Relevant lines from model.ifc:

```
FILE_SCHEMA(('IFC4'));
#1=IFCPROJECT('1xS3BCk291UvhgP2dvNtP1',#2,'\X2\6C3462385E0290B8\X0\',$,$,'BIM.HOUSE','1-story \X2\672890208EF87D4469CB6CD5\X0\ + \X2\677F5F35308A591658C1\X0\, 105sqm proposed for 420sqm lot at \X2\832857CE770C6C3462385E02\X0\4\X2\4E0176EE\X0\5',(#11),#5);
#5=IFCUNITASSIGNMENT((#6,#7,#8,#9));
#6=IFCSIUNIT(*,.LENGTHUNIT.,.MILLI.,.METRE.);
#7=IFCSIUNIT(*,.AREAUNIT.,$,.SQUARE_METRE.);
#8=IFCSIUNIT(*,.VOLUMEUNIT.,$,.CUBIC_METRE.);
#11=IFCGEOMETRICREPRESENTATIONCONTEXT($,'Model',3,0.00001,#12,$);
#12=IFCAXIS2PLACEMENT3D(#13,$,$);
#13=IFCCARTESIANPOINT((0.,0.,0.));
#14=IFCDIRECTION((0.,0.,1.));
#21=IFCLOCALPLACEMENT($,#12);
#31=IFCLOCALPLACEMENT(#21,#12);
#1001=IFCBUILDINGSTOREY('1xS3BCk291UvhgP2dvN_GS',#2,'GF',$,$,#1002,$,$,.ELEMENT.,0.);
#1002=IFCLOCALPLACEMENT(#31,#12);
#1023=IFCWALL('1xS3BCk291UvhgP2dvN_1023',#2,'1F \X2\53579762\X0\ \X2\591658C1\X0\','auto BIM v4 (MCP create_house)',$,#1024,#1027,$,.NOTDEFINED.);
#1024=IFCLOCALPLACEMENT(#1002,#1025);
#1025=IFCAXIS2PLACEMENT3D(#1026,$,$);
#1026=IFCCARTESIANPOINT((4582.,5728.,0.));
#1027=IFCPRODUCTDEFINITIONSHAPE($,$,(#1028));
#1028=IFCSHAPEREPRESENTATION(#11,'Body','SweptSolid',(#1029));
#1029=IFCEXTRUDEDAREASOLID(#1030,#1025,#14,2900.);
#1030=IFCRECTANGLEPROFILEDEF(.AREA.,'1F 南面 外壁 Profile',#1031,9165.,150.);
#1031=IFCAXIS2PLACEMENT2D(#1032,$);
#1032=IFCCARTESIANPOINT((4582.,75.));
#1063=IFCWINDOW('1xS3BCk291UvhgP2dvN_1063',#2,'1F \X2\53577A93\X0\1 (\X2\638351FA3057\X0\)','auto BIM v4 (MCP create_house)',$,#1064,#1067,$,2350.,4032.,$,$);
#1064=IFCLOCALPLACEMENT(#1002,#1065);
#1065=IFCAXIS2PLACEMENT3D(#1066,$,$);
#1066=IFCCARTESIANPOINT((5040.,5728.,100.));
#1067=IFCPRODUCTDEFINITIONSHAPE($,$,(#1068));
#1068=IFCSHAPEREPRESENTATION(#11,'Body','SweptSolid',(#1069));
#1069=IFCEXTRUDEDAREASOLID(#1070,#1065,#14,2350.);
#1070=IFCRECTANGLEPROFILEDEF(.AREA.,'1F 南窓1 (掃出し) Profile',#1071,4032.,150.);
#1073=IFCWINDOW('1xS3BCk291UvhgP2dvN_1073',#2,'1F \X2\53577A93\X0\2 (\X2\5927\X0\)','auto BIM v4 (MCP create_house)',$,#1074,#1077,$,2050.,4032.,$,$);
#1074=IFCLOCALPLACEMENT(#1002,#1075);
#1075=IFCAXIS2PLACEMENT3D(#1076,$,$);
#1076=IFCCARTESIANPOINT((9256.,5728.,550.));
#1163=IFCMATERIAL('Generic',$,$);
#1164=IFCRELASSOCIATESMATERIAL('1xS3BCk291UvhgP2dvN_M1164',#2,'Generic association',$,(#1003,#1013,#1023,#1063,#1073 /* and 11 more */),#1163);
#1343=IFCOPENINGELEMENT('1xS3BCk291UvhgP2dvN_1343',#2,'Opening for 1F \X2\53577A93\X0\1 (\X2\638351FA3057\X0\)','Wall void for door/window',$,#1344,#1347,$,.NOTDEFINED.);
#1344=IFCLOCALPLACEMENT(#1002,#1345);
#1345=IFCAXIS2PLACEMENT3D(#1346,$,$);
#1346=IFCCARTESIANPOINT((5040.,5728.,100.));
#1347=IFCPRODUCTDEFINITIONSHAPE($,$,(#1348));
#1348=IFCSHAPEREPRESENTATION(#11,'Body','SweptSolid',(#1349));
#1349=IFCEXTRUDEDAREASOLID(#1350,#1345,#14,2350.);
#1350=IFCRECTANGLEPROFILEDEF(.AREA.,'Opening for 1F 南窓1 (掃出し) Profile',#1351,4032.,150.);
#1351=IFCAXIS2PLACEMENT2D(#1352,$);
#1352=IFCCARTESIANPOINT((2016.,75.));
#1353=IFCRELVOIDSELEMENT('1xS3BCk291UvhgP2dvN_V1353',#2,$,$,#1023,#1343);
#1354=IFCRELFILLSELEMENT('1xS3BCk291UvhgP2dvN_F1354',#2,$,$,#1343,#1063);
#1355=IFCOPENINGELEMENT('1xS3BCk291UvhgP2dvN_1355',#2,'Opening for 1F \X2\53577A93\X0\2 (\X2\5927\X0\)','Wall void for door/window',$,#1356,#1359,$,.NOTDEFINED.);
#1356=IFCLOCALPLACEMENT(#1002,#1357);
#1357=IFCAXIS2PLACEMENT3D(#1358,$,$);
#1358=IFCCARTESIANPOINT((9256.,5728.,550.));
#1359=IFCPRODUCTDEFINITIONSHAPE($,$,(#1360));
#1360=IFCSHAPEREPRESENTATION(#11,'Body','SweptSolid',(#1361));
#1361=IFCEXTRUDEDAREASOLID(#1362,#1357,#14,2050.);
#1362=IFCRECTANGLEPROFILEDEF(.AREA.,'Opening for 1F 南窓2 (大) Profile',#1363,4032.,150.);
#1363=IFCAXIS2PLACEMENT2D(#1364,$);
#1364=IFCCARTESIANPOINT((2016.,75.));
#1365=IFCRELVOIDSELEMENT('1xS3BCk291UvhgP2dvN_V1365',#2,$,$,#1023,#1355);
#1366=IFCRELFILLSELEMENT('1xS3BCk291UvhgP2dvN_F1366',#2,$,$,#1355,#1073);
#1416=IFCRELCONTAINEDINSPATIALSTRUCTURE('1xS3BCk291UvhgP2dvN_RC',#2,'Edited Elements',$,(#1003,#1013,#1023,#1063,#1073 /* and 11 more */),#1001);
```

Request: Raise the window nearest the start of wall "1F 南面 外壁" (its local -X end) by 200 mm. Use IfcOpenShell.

```python
import numpy as np
import ifcopenshell
import ifcopenshell.api.geometry
import ifcopenshell.util.placement
import ifcopenshell.util.unit

model = ifcopenshell.open("model.ifc")
unit_scale = ifcopenshell.util.unit.calculate_unit_scale(model)

window = model.by_id(1063)
opening = window.FillsVoids[0].RelatingOpeningElement
dz = 0.2 / unit_scale

shift = np.array([0.0, 0.0, dz])
# The window is not placed relative to its opening, so move both.
for product in (opening, window):
    matrix = ifcopenshell.util.placement.get_local_placement(product.ObjectPlacement)
    matrix[:3, 3] += shift
    ifcopenshell.api.geometry.edit_object_placement(model, product=product, matrix=matrix, is_si=False)

print(f"moved by {dz * unit_scale:+.3f} m")

model.write("model_rev.ifc")
```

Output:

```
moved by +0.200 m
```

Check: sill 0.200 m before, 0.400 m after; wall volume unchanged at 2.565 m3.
